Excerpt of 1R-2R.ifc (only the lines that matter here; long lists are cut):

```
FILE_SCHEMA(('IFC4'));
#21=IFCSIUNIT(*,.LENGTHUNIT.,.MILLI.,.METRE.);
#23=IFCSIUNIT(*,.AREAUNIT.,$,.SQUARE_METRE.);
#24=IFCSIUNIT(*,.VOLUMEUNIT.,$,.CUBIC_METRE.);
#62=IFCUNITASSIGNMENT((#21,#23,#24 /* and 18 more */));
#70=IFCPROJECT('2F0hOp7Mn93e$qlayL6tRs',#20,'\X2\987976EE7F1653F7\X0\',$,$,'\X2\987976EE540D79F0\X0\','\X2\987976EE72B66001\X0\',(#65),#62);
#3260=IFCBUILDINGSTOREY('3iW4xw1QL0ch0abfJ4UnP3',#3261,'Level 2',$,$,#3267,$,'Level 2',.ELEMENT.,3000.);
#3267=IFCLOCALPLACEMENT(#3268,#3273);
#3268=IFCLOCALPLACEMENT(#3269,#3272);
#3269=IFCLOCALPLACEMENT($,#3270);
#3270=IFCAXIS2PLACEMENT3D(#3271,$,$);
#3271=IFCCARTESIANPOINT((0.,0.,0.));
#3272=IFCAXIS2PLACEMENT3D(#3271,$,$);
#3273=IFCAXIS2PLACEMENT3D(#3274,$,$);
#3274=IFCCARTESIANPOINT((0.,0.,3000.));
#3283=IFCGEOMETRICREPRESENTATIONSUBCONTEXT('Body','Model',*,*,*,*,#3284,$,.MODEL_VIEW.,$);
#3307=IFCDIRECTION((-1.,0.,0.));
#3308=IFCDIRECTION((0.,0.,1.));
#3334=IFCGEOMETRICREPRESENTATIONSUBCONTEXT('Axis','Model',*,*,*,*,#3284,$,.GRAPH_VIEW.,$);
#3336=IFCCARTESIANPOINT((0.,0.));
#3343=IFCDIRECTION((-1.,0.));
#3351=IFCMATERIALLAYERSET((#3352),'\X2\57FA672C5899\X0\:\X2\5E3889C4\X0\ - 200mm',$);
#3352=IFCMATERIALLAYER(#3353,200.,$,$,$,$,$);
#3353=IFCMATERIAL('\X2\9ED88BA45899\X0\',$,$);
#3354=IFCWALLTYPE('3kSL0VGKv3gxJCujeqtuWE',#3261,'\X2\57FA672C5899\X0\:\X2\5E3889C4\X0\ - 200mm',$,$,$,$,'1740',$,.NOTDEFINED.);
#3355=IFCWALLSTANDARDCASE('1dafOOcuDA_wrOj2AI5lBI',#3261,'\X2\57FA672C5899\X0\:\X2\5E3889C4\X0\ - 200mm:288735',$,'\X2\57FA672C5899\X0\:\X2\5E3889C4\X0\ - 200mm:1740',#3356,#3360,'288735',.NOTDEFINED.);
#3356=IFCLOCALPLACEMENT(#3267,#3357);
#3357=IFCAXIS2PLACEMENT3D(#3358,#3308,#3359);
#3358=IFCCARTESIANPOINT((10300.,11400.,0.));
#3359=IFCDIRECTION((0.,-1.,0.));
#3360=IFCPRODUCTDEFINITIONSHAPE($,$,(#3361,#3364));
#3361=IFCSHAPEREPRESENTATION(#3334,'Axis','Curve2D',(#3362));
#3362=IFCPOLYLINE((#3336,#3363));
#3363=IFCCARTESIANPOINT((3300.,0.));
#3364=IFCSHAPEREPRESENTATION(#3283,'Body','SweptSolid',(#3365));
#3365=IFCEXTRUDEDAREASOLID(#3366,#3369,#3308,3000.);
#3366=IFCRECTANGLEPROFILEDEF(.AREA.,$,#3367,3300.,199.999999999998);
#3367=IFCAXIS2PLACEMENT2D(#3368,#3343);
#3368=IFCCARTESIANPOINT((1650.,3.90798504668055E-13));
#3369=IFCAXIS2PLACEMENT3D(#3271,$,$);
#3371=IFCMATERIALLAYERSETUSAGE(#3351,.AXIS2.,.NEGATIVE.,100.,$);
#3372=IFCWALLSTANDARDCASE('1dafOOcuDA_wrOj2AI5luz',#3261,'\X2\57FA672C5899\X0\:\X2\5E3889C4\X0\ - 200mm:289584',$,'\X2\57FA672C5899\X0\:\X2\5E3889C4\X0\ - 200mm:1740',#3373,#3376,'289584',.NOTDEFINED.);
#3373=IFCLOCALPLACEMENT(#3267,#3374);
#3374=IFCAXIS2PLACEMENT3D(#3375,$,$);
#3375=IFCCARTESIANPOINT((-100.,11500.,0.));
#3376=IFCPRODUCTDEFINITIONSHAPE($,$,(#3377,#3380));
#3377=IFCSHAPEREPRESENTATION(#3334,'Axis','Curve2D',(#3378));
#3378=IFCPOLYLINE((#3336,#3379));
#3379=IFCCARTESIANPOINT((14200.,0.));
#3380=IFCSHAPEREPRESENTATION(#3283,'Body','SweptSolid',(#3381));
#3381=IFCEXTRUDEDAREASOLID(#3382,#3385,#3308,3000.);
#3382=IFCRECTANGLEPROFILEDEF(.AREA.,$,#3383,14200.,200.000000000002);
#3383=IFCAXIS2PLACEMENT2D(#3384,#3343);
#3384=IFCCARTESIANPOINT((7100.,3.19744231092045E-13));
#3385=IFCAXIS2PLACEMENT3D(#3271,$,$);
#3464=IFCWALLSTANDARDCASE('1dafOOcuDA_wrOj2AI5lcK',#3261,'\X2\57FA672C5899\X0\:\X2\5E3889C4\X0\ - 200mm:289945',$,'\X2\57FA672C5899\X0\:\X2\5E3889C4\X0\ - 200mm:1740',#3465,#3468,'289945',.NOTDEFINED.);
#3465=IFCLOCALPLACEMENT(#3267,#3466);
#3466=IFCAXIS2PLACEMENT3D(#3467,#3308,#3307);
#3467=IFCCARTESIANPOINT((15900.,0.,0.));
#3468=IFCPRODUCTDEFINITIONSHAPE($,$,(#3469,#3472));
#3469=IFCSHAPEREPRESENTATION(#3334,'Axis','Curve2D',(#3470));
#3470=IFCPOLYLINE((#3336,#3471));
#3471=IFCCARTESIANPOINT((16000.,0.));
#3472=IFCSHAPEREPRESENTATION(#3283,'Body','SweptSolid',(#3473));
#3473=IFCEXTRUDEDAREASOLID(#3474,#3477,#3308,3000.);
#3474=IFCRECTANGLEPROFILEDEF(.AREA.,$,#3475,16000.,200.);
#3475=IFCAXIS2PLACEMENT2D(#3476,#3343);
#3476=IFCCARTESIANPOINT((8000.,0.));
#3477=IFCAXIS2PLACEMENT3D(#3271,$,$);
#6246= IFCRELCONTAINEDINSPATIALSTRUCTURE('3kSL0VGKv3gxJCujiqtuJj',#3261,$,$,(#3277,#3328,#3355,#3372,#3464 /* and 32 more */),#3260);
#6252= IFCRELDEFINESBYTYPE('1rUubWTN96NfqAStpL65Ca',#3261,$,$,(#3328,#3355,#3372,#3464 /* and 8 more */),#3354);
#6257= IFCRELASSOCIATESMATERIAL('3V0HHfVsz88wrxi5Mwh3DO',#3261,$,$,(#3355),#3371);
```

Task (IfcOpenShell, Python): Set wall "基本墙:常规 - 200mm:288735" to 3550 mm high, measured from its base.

```python
import ifcopenshell
import ifcopenshell.geom
import ifcopenshell.util.representation
import ifcopenshell.util.shape

model = ifcopenshell.open("1R-2R.ifc")
settings = ifcopenshell.geom.settings()


def volume(element):
    """Net volume in cubic metres, openings subtracted."""
    shape = ifcopenshell.geom.create_shape(settings, element)
    return ifcopenshell.util.shape.get_volume(shape.geometry)


wall = model.by_guid("1dafOOcuDA_wrOj2AI5lBI")
before = volume(wall)

body = ifcopenshell.util.representation.get_representation(wall, "Model", "Body")
solid = body.Items[0]
old_height = solid.Depth
solid.Depth = 3550.0
after = volume(wall)

print(f"height {old_height:g} -> {solid.Depth:g}, volume {before:.3f} -> {after:.3f} m3")

model.write("1R-2R_edited.ifc")
```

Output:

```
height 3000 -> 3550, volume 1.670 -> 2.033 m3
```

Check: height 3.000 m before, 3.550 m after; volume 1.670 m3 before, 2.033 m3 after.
